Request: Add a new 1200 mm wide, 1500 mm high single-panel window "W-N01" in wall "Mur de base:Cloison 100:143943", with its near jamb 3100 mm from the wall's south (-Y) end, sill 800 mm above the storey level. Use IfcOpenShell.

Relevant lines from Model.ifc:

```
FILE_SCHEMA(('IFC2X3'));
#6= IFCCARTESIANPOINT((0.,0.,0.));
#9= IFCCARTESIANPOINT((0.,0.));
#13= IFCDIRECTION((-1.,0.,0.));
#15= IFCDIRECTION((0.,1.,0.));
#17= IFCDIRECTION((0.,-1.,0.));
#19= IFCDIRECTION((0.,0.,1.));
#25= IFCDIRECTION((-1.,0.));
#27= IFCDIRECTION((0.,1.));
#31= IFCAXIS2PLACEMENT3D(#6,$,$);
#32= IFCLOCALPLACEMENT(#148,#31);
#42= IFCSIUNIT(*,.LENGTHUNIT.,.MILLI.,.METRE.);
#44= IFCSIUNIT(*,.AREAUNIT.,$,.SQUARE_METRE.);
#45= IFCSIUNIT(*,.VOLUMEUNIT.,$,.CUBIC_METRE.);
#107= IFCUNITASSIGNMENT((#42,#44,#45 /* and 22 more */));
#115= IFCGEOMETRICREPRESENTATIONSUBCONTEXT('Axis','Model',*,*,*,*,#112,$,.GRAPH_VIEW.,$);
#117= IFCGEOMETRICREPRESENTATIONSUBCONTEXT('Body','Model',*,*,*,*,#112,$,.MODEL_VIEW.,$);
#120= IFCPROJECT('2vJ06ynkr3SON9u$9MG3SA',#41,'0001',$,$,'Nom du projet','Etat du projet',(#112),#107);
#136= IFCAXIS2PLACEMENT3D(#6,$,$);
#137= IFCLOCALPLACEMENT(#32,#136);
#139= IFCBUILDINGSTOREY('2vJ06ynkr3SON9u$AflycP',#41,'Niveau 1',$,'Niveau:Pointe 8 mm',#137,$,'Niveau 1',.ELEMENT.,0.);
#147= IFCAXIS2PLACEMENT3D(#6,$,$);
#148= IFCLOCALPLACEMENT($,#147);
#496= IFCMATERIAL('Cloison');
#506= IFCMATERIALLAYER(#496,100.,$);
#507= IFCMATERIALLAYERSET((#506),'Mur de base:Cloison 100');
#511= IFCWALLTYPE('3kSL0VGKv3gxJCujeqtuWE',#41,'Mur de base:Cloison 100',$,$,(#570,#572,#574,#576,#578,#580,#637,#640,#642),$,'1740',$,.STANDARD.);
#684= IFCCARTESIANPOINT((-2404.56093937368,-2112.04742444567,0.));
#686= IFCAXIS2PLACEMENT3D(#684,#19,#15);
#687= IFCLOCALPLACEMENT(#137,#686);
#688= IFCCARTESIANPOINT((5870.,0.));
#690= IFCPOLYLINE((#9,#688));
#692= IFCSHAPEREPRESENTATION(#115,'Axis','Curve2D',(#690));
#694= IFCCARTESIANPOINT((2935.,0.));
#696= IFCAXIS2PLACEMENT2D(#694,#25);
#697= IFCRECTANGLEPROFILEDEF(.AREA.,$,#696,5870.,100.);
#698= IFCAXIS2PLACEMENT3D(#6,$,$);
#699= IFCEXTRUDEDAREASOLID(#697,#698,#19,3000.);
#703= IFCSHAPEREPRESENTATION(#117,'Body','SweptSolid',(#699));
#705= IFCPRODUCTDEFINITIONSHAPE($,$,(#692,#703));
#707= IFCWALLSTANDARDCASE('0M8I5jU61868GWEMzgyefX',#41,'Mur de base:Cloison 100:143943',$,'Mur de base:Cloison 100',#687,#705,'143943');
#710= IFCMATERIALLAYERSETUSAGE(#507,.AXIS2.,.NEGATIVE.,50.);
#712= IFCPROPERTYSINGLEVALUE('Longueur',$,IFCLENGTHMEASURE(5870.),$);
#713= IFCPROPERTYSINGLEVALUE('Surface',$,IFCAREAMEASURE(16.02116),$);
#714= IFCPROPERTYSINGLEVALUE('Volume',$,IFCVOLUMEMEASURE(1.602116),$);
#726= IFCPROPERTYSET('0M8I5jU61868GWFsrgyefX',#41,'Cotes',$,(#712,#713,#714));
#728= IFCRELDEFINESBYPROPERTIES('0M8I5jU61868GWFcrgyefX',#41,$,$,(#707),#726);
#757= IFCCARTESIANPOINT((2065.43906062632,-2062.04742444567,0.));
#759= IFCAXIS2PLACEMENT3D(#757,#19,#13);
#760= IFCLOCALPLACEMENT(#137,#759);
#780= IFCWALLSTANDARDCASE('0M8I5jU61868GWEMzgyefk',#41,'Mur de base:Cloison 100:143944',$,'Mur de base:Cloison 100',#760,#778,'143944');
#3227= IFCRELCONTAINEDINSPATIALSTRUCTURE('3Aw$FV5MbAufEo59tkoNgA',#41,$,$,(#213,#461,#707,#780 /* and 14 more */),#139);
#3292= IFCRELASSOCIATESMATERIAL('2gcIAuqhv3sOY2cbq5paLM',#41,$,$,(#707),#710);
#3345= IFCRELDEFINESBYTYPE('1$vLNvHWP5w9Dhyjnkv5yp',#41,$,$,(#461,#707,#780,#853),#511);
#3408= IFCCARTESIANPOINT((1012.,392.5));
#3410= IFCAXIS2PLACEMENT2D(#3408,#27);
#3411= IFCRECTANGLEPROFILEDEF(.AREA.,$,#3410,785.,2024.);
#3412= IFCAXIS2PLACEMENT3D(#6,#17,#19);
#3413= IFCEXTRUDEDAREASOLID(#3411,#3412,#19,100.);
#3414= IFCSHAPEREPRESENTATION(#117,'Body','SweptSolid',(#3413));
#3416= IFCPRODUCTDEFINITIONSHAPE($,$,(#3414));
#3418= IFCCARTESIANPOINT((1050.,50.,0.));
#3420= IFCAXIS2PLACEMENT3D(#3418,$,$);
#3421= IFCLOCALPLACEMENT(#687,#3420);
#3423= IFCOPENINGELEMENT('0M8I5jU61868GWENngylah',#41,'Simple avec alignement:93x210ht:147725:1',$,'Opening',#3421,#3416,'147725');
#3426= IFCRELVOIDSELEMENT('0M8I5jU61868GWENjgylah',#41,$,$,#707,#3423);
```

```python
import numpy as np
import ifcopenshell
import ifcopenshell.api.feature
import ifcopenshell.api.geometry
import ifcopenshell.api.pset
import ifcopenshell.api.root
import ifcopenshell.api.spatial
import ifcopenshell.api.type
import ifcopenshell.geom
import ifcopenshell.util.element
import ifcopenshell.util.placement
import ifcopenshell.util.representation
import ifcopenshell.util.shape
import ifcopenshell.util.unit

model = ifcopenshell.open("Model.ifc")
unit_scale = ifcopenshell.util.unit.calculate_unit_scale(model)
area_scale = ifcopenshell.util.unit.calculate_unit_scale(model, "AREAUNIT")
volume_scale = ifcopenshell.util.unit.calculate_unit_scale(model, "VOLUMEUNIT")
settings = ifcopenshell.geom.settings()


def volume(element):
    """Net volume in cubic metres, openings subtracted."""
    shape = ifcopenshell.geom.create_shape(settings, element)
    return ifcopenshell.util.shape.get_volume(shape.geometry)


wall = model.by_id(707)
storey = ifcopenshell.util.element.get_container(wall, ifc_class="IfcBuildingStorey")
context = ifcopenshell.util.representation.get_context(model, "Model", "Body", "MODEL_VIEW")
before = volume(wall)

width, height, from_end, sill = 1.2, 1.5, 3.1, 0.8  # metres

# The wall runs along its own X axis, and the end named is its -X end.
wall_shape = ifcopenshell.geom.create_shape(settings, wall)
x, y, z = ifcopenshell.util.shape.get_vertices(wall_shape.geometry).T
start = x.min() + from_end
face, thickness = float(y.min()), float(y.max() - y.min())
wall_matrix = ifcopenshell.util.placement.get_local_placement(wall.ObjectPlacement)
level = ifcopenshell.util.placement.get_local_placement(storey.ObjectPlacement)[2, 3]


def in_wall(x, y):
    """Placement at x, y metres in the wall's axes, at sill height."""
    matrix = wall_matrix.copy()
    matrix[:, 3] = wall_matrix @ np.array([x / unit_scale, y / unit_scale, 0.0, 1.0])
    matrix[2, 3] = level + sill / unit_scale
    return matrix


# Opening: a box that overshoots both wall faces by 50 mm.
opening = ifcopenshell.api.root.create_entity(model, ifc_class="IfcOpeningElement")
box = ifcopenshell.api.geometry.add_wall_representation(
    model, context=context, length=width, height=height, thickness=thickness + 0.1
)
ifcopenshell.api.geometry.assign_representation(model, product=opening, representation=box)
ifcopenshell.api.geometry.edit_object_placement(model, product=opening, matrix=in_wall(start, face - 0.05), is_si=False)
ifcopenshell.api.feature.add_feature(model, feature=opening, element=wall)

window = ifcopenshell.api.root.create_entity(model, ifc_class="IfcWindow", name="W-N01")
window.OverallWidth, window.OverallHeight = width / unit_scale, height / unit_scale
body = ifcopenshell.api.geometry.add_window_representation(
    model,
    context=context,
    overall_width=window.OverallWidth,
    overall_height=window.OverallHeight,
    partition_type="SINGLE_PANEL",
)
ifcopenshell.api.geometry.assign_representation(model, product=window, representation=body)
ifcopenshell.api.spatial.assign_container(model, products=[window], relating_structure=storey)
fills = ifcopenshell.api.feature.add_filling(model, opening=opening, element=window)
fills.OwnerHistory = window.OwnerHistory  # required in IFC2X3

# IFC2X3 keeps the operation on the window style.
style = ifcopenshell.api.root.create_entity(model, ifc_class="IfcWindowStyle", name="W-N01")
style.OperationType, style.ConstructionType = "SINGLE_PANEL", "NOTDEFINED"
style.ParameterTakesPrecedence = style.Sizeable = False
ifcopenshell.api.type.assign_type(model, related_objects=[window], relating_type=style)

# Centre the window in the wall's thickness.
ifcopenshell.api.geometry.edit_object_placement(model, product=window, matrix=in_wall(start, face), is_si=False)
window_shape = ifcopenshell.geom.create_shape(settings, window)
depth = ifcopenshell.util.shape.get_vertices(window_shape.geometry)[:, 1]
offset = face + thickness / 2 - (depth.min() + depth.max()) / 2
ifcopenshell.api.geometry.edit_object_placement(model, product=window, matrix=in_wall(start, offset), is_si=False)

after = volume(wall)

# Update the wall's stored quantities.
pset = model.by_id(ifcopenshell.util.element.get_pset(wall, "Cotes", should_inherit=False)["id"])
ifcopenshell.api.pset.edit_pset(model, pset=pset, properties={
    "Surface": model.create_entity("IfcAreaMeasure", after / thickness / area_scale),
    "Volume": model.create_entity("IfcVolumeMeasure", after / volume_scale),
})

print(f"wall volume {before:.3f} -> {after:.3f} m3")

model.write("Model_rev.ifc")
```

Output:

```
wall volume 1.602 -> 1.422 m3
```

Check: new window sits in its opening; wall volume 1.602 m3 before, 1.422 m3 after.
